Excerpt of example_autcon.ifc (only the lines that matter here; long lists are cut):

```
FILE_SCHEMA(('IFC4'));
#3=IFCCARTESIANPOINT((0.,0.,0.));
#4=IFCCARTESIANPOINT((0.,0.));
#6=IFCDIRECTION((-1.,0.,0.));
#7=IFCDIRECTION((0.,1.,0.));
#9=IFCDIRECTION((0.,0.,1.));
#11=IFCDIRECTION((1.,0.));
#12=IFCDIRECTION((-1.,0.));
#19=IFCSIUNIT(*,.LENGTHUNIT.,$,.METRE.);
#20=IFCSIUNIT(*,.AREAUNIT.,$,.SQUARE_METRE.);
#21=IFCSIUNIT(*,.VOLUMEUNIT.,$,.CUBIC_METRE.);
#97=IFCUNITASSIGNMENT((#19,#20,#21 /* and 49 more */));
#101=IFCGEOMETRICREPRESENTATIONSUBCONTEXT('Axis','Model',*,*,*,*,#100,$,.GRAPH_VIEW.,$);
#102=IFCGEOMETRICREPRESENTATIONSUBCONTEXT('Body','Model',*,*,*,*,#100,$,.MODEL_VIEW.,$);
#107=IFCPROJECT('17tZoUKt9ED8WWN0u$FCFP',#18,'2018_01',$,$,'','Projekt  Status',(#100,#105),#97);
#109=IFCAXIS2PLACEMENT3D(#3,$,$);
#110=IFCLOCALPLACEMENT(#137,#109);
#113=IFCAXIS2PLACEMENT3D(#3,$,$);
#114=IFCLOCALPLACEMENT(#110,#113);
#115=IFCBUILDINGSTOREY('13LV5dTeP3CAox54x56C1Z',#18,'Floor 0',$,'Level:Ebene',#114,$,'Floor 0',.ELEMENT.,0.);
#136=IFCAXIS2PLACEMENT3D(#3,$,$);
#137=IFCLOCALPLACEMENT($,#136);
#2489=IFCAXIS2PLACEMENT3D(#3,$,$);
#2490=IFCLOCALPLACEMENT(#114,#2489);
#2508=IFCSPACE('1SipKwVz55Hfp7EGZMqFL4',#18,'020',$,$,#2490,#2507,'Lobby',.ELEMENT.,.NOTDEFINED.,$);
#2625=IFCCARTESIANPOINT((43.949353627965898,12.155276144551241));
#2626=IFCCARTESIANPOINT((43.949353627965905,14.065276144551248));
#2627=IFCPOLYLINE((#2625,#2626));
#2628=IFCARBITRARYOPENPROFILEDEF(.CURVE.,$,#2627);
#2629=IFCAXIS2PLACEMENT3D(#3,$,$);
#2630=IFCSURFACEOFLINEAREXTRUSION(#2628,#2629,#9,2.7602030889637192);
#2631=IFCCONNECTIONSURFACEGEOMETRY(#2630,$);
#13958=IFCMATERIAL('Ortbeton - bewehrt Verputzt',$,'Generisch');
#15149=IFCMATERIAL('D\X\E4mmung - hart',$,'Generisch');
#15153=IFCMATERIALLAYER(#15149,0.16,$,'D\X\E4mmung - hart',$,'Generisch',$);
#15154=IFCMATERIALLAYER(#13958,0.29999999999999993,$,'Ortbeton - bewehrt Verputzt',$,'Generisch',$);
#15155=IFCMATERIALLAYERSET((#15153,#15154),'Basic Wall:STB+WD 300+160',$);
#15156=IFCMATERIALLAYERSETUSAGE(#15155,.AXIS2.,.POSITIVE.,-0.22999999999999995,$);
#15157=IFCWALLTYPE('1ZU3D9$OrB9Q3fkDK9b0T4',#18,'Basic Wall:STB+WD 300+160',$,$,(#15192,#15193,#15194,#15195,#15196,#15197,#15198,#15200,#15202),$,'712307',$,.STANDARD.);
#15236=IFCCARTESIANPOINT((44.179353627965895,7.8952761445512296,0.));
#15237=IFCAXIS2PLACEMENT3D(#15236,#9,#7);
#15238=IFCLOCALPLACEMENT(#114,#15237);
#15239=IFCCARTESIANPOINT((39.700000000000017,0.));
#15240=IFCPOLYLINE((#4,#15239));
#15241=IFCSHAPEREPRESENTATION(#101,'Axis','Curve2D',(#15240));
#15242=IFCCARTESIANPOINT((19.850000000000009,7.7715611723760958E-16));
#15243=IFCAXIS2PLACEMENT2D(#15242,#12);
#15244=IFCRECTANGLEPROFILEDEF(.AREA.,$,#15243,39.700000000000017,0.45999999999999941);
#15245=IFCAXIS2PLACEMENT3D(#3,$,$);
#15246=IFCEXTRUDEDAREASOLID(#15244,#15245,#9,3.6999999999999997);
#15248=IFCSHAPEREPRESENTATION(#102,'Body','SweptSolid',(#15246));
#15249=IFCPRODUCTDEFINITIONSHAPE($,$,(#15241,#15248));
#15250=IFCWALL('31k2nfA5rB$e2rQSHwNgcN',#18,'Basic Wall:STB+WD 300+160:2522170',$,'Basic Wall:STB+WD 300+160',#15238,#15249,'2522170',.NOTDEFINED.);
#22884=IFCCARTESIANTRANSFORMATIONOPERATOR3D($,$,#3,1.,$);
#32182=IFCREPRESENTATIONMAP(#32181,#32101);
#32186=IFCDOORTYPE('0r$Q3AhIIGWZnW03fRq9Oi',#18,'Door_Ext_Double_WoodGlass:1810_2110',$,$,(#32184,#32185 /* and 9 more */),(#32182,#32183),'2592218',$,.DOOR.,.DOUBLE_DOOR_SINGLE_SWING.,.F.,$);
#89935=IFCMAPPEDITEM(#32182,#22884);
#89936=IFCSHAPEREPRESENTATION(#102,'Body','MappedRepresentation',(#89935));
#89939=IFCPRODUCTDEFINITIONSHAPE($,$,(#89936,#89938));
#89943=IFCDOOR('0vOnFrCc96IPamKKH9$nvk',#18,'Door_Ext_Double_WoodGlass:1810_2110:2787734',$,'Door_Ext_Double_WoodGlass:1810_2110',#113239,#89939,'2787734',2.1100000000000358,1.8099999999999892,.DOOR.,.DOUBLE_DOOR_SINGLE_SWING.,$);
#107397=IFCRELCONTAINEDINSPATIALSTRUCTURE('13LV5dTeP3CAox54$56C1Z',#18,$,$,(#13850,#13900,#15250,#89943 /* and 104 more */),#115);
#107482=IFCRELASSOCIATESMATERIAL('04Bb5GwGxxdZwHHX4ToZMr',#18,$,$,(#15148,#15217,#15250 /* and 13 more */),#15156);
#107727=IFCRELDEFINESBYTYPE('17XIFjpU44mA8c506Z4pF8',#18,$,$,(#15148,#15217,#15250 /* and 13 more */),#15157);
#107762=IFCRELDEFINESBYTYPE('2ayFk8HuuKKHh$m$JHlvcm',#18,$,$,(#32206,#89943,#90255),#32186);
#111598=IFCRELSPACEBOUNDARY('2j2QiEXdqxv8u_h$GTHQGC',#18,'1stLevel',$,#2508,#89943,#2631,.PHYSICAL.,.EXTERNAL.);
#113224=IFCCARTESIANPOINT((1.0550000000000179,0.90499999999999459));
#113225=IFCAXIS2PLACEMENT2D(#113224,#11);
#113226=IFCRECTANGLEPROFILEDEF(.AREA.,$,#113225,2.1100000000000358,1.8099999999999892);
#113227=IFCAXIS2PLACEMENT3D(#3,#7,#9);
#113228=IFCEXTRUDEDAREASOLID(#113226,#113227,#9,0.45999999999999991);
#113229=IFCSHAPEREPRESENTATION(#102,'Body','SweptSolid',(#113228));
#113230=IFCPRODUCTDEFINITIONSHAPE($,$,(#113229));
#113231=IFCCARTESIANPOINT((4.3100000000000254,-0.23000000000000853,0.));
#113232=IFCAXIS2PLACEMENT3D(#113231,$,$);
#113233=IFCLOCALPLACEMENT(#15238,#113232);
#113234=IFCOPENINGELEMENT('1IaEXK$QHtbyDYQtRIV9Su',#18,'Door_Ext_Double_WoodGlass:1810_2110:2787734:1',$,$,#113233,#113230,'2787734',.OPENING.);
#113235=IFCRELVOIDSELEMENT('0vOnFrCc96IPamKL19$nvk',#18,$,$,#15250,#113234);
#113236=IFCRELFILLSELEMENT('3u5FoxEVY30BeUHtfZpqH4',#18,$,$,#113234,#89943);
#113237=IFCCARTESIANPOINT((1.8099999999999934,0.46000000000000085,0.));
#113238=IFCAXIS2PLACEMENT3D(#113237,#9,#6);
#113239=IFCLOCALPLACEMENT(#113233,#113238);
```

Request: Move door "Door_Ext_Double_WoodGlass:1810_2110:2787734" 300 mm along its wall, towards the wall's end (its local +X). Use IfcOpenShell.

```python
import numpy as np
import ifcopenshell
import ifcopenshell.api.geometry
import ifcopenshell.util.placement

model = ifcopenshell.open("example_autcon.ifc")

door = model.by_id(89943)
opening = door.FillsVoids[0].RelatingOpeningElement
wall = opening.VoidsElements[0].RelatingBuildingElement

wall_matrix = ifcopenshell.util.placement.get_local_placement(wall.ObjectPlacement)
shift = wall_matrix[:3, 0] * 0.3
before = ifcopenshell.util.placement.get_local_placement(door.ObjectPlacement)[:3, 3].copy()

# The door is placed relative to its opening, so it follows when the opening moves.
matrix = ifcopenshell.util.placement.get_local_placement(opening.ObjectPlacement)
matrix[:3, 3] += shift
ifcopenshell.api.geometry.edit_object_placement(
    model, product=opening, matrix=matrix, is_si=False, should_transform_children=True
)

# Space boundary surfaces are stored in each space's coordinates; move them too.
for rel in door.ProvidesBoundaries:
    if not rel.ConnectionGeometry:
        continue
    surface = rel.ConnectionGeometry.SurfaceOnRelatingElement
    space_matrix = ifcopenshell.util.placement.get_local_placement(rel.RelatingSpace.ObjectPlacement)
    point = np.array(surface.Position.Location.Coordinates) + space_matrix[:3, :3].T @ shift
    surface.Position = model.createIfcAxis2Placement3D(
        model.createIfcCartesianPoint(point.tolist()), surface.Position.Axis, surface.Position.RefDirection
    )

after = ifcopenshell.util.placement.get_local_placement(door.ObjectPlacement)[:3, 3]
print("door moved by", (after - before).round(3) + 0.0)

model.write("example_autcon_updated.ifc")
```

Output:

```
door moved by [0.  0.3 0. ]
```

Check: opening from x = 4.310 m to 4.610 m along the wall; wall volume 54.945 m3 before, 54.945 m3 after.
